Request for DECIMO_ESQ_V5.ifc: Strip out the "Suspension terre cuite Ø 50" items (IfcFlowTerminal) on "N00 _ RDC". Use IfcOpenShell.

First a look at what the model holds.

```python
import ifcopenshell
import ifcopenshell.util.element

model = ifcopenshell.open("DECIMO_ESQ_V5.ifc")
print(model.schema)
storey = next(s for s in model.by_type("IfcBuildingStorey") if s.Name == "N00 _ RDC")
terminals = [e for e in ifcopenshell.util.element.get_decomposition(storey) if e.is_a("IfcFlowTerminal")]
seen = {}
for e in terminals:
    element_type = ifcopenshell.util.element.get_type(e)
    name = element_type.Name if element_type not in (None, e) else None
    seen[name] = seen.get(name, 0) + 1
for name, count in sorted(seen.items(), key=str):
    print(count, "x", name)
```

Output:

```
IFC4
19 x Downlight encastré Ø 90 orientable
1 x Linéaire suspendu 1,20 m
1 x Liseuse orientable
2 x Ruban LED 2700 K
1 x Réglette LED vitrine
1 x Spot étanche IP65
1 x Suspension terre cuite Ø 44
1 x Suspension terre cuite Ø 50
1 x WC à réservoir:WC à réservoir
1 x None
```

```python
import ifcopenshell
import ifcopenshell.api.root
import ifcopenshell.util.element

model = ifcopenshell.open("DECIMO_ESQ_V5.ifc")

storey = next(s for s in model.by_type("IfcBuildingStorey") if s.Name == "N00 _ RDC")
terminals = [e for e in ifcopenshell.util.element.get_decomposition(storey) if e.is_a("IfcFlowTerminal")]
targets = [e for e in terminals if (t := ifcopenshell.util.element.get_type(e)) not in (None, e) and t.Name == "Suspension terre cuite Ø 50"]

for e in targets:
    ifcopenshell.api.root.remove_product(model, product=e)
print(len(targets), "removed")

model.write("DECIMO_ESQ_V5_v2.ifc")
```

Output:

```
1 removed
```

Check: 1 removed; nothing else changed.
